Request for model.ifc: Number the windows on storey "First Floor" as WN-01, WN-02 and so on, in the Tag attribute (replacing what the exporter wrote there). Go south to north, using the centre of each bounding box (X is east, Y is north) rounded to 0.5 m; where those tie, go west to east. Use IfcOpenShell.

First a look at what the model holds.

```python
import ifcopenshell
import ifcopenshell.util.element
import ifcopenshell.util.placement

model = ifcopenshell.open("model.ifc")
print(model.schema)
storey = next(s for s in model.by_type("IfcBuildingStorey") if s.Name == "First Floor")
windows = [e for e in ifcopenshell.util.element.get_decomposition(storey) if e.is_a("IfcWindow")]
for e in sorted(windows, key=lambda e: e.id()):
    origin = ifcopenshell.util.placement.get_local_placement(e.ObjectPlacement)[:3, 3]
    print(e.id(), e.Tag, e.Name, origin.round(2) + 0.0, sep=" | ")
```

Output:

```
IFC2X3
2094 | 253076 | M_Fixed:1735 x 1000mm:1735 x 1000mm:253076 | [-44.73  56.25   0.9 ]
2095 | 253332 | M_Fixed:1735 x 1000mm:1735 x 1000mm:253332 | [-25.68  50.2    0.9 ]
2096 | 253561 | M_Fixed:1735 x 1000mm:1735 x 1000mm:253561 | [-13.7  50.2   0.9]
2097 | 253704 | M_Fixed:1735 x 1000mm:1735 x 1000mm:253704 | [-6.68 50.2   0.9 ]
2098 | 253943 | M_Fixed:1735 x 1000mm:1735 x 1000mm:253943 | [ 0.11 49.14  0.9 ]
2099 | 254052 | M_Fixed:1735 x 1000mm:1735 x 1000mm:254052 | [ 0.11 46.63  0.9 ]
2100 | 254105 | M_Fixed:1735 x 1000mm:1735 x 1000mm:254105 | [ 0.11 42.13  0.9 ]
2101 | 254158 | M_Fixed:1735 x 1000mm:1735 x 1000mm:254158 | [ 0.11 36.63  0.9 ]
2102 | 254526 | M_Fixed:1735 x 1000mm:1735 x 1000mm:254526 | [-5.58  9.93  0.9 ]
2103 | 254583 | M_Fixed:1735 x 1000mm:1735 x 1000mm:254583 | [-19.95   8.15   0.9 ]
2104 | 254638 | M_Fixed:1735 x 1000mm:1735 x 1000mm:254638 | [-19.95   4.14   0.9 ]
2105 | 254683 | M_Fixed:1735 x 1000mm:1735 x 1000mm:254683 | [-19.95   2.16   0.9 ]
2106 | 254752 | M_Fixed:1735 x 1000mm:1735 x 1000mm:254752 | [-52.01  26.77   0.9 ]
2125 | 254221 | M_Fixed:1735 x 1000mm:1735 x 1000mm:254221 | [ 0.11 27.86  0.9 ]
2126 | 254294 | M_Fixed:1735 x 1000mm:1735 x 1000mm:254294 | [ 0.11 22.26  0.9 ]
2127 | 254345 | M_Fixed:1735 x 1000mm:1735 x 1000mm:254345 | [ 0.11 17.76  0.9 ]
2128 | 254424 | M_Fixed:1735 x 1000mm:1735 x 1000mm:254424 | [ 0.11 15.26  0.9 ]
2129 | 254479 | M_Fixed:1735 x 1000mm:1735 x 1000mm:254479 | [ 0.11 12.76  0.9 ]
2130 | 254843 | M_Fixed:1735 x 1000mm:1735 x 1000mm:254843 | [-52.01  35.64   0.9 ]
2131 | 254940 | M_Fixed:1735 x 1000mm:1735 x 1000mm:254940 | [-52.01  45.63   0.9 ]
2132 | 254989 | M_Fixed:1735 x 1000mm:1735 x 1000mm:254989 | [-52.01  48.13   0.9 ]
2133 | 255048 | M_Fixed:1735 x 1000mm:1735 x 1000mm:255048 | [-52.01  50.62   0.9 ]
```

```python
import ifcopenshell
import ifcopenshell.geom
import ifcopenshell.util.element
import ifcopenshell.util.shape

model = ifcopenshell.open("model.ifc")
settings = ifcopenshell.geom.settings()
settings.set("use-world-coords", True)


def centre(element):
    shape = ifcopenshell.geom.create_shape(settings, element)
    return ifcopenshell.util.shape.get_bbox_centroid(shape.geometry)


storey = next(s for s in model.by_type("IfcBuildingStorey") if s.Name == "First Floor")
windows = [e for e in ifcopenshell.util.element.get_decomposition(storey) if e.is_a("IfcWindow")]

# Insertion points can sit at a corner or the storey origin, so sort by the geometry (in metres).
centres = {e: centre(e) for e in windows}
windows.sort(key=lambda e: (round(centres[e][1] / 0.5), centres[e][0]))

for i, e in enumerate(windows, start=1):
    number = f"WN-{i:02d}"
    e.Tag = number
    print(e.id(), number)

model.write("model_updated.ifc")
```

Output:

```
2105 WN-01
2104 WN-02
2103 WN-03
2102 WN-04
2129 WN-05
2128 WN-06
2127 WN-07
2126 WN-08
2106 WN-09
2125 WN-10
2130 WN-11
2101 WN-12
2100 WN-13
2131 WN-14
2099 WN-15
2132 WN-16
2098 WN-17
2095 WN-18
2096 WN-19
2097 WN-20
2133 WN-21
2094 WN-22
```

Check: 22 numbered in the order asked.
